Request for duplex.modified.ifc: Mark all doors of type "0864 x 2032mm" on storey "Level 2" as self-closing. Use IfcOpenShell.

First a look at what the model holds.

```python
import ifcopenshell
import ifcopenshell.util.element

model = ifcopenshell.open("duplex.modified.ifc")
print(model.schema)
storey = next(s for s in model.by_type("IfcBuildingStorey") if s.Name == "Level 2")
doors = [e for e in ifcopenshell.util.element.get_decomposition(storey) if e.is_a("IfcDoor")]
seen = {}
for e in doors:
    element_type = ifcopenshell.util.element.get_type(e)
    key = (element_type.Name if element_type != e and element_type else None, ifcopenshell.util.element.get_pset(e, "Pset_DoorCommon", "SelfClosing"))
    seen[key] = seen.get(key, 0) + 1
for (name, value), count in sorted(seen.items(), key=str):
    print(count, "x", name, "|", value)
```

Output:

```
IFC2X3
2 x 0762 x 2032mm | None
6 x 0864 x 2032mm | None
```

```python
import ifcopenshell
import ifcopenshell.api.pset
import ifcopenshell.util.element

model = ifcopenshell.open("duplex.modified.ifc")

storey = next(s for s in model.by_type("IfcBuildingStorey") if s.Name == "Level 2")
doors = [e for e in ifcopenshell.util.element.get_decomposition(storey) if e.is_a("IfcDoor")]

count = 0
for e in doors:
    element_type = ifcopenshell.util.element.get_type(e)
    if element_type in (None, e) or element_type.Name != "0864 x 2032mm":
        continue
    # add_pset returns the element's existing set when there is one.
    pset = ifcopenshell.api.pset.add_pset(model, product=e, name="Pset_DoorCommon")
    ifcopenshell.api.pset.edit_pset(model, pset=pset, properties={"SelfClosing": True})
    count += 1

print(count, "doors updated")

model.write("duplex.modified_edited.ifc")
```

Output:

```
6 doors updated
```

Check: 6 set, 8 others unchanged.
